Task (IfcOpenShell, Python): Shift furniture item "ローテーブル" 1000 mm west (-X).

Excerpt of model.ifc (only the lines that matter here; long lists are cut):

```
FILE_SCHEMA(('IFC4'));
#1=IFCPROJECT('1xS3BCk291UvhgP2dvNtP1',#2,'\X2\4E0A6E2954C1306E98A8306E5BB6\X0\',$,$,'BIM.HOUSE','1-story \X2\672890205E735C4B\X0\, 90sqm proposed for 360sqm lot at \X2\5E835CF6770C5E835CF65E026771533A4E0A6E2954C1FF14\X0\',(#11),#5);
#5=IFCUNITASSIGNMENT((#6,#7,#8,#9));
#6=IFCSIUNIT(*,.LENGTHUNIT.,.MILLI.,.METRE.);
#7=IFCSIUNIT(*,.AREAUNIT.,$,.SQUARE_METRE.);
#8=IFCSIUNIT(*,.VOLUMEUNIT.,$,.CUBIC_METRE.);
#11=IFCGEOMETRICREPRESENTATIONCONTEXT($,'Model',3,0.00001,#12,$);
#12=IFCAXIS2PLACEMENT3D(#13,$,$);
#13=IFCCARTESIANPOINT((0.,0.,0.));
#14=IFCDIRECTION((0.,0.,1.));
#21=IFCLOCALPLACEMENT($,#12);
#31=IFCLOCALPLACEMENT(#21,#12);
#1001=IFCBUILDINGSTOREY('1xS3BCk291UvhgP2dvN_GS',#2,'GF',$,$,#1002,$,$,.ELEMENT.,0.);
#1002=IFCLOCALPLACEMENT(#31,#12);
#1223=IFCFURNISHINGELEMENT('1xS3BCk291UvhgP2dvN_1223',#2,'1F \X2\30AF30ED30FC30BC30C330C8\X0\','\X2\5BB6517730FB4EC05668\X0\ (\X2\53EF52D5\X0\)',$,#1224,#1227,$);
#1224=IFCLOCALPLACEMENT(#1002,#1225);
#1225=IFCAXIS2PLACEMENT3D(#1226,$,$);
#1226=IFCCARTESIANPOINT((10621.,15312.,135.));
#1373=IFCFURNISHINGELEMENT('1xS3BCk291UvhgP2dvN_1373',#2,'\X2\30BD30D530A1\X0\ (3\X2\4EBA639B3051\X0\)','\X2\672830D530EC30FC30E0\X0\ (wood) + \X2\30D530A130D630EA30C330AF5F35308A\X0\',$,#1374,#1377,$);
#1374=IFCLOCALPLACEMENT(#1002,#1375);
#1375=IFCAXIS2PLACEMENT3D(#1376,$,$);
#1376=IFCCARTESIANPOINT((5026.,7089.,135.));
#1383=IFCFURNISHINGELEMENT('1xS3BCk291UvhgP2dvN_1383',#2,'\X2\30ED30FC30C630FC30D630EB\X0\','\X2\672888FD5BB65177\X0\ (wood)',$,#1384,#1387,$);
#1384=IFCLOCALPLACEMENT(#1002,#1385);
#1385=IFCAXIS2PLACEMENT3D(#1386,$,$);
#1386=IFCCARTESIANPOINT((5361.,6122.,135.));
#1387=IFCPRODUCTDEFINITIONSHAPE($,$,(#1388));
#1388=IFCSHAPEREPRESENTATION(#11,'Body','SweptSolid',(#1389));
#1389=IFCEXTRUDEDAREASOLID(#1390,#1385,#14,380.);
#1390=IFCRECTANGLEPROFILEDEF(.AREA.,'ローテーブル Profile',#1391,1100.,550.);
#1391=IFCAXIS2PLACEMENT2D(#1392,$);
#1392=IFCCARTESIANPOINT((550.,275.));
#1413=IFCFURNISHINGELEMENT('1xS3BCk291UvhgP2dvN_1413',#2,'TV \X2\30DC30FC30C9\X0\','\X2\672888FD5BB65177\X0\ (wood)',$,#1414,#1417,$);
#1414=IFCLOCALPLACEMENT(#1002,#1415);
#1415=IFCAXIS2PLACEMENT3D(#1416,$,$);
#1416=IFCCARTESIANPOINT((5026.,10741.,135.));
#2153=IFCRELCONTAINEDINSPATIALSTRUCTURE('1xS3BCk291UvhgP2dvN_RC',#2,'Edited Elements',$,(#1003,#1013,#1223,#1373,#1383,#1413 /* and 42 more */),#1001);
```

```python
import ifcopenshell
import ifcopenshell.api.geometry
import ifcopenshell.util.placement
import ifcopenshell.util.unit

model = ifcopenshell.open("model.ifc")
unit_scale = ifcopenshell.util.unit.calculate_unit_scale(model)

item = model.by_guid("1xS3BCk291UvhgP2dvN_1383")
matrix = ifcopenshell.util.placement.get_local_placement(item.ObjectPlacement)
matrix[0, 3] -= 1 / unit_scale
ifcopenshell.api.geometry.edit_object_placement(model, product=item, matrix=matrix, is_si=False)

print(ifcopenshell.util.placement.get_local_placement(item.ObjectPlacement).round(3) + 0.0)

model.write("model-out.ifc")
```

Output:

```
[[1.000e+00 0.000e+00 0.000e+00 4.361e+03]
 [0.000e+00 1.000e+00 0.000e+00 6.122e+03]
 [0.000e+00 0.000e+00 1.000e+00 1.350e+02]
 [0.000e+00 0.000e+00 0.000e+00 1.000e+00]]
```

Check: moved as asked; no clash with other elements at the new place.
